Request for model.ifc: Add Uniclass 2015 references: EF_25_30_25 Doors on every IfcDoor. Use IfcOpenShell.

First a look at what the model holds.

```python
import ifcopenshell

model = ifcopenshell.open("model.ifc")
print(model.schema)
print("classifications:", [c.Name for c in model.by_type("IfcClassification")])
for ifc_class in ("IfcDoor", "IfcRoof", "IfcStair", "IfcWall", "IfcWindow"):
    print(ifc_class, len(model.by_type(ifc_class)))
```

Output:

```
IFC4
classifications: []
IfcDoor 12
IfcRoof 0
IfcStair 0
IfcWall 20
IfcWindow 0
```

```python
import ifcopenshell
import ifcopenshell.api.classification

model = ifcopenshell.open("model.ifc")

system = ifcopenshell.api.classification.add_classification(model, classification="Uniclass 2015")

codes = {
    "IfcDoor": ("EF_25_30_25", "Doors"),
}
for ifc_class, (code, name) in codes.items():
    products = model.by_type(ifc_class)
    ifcopenshell.api.classification.add_reference(
        model, products=products, classification=system, identification=code, name=name
    )
    print(code, len(products))

model.write("model_rev.ifc")
```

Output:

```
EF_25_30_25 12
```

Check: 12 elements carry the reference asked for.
